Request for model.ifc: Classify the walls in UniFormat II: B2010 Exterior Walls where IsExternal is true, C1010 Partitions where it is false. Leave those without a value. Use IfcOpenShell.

First a look at what the model holds.

```python
import ifcopenshell
import ifcopenshell.util.element

model = ifcopenshell.open("model.ifc")
print(model.schema)
print("classifications:", [c.Name for c in model.by_type("IfcClassification")])
values = [ifcopenshell.util.element.get_pset(e, "Pset_WallCommon", "IsExternal") for e in model.by_type("IfcWall")]
for value in (True, False, None):
    print("IsExternal", value, values.count(value))
```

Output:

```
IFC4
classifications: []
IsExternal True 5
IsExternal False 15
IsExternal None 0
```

```python
import ifcopenshell
import ifcopenshell.api.classification
import ifcopenshell.util.element

model = ifcopenshell.open("model.ifc")

system = ifcopenshell.api.classification.add_classification(model, classification="UniFormat II")

walls = model.by_type("IfcWall")
external = {e: ifcopenshell.util.element.get_pset(e, "Pset_WallCommon", "IsExternal") for e in walls}
for flag, code, name in ((True, "B2010", "Exterior Walls"), (False, "C1010", "Partitions")):
    products = [e for e in walls if external[e] is flag]
    ifcopenshell.api.classification.add_reference(
        model, products=products, classification=system, identification=code, name=name
    )
    print(code, len(products))

model.write("model_updated.ifc")
```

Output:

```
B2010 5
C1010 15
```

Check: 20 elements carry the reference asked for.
